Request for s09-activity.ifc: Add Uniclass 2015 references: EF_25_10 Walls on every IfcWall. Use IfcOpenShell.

First a look at what the model holds.

```python
import ifcopenshell

model = ifcopenshell.open("s09-activity.ifc")
print(model.schema)
print("classifications:", [c.Name for c in model.by_type("IfcClassification")])
for ifc_class in ("IfcDoor", "IfcRoof", "IfcStair", "IfcWall", "IfcWindow"):
    print(ifc_class, len(model.by_type(ifc_class)))
```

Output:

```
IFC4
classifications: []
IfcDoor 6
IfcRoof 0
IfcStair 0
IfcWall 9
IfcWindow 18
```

```python
import ifcopenshell
import ifcopenshell.api.classification

model = ifcopenshell.open("s09-activity.ifc")

system = ifcopenshell.api.classification.add_classification(model, classification="Uniclass 2015")

codes = {
    "IfcWall": ("EF_25_10", "Walls"),
}
for ifc_class, (code, name) in codes.items():
    products = model.by_type(ifc_class)
    ifcopenshell.api.classification.add_reference(
        model, products=products, classification=system, identification=code, name=name
    )
    print(code, len(products))

model.write("s09-activity-out.ifc")
```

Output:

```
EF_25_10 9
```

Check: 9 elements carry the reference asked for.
